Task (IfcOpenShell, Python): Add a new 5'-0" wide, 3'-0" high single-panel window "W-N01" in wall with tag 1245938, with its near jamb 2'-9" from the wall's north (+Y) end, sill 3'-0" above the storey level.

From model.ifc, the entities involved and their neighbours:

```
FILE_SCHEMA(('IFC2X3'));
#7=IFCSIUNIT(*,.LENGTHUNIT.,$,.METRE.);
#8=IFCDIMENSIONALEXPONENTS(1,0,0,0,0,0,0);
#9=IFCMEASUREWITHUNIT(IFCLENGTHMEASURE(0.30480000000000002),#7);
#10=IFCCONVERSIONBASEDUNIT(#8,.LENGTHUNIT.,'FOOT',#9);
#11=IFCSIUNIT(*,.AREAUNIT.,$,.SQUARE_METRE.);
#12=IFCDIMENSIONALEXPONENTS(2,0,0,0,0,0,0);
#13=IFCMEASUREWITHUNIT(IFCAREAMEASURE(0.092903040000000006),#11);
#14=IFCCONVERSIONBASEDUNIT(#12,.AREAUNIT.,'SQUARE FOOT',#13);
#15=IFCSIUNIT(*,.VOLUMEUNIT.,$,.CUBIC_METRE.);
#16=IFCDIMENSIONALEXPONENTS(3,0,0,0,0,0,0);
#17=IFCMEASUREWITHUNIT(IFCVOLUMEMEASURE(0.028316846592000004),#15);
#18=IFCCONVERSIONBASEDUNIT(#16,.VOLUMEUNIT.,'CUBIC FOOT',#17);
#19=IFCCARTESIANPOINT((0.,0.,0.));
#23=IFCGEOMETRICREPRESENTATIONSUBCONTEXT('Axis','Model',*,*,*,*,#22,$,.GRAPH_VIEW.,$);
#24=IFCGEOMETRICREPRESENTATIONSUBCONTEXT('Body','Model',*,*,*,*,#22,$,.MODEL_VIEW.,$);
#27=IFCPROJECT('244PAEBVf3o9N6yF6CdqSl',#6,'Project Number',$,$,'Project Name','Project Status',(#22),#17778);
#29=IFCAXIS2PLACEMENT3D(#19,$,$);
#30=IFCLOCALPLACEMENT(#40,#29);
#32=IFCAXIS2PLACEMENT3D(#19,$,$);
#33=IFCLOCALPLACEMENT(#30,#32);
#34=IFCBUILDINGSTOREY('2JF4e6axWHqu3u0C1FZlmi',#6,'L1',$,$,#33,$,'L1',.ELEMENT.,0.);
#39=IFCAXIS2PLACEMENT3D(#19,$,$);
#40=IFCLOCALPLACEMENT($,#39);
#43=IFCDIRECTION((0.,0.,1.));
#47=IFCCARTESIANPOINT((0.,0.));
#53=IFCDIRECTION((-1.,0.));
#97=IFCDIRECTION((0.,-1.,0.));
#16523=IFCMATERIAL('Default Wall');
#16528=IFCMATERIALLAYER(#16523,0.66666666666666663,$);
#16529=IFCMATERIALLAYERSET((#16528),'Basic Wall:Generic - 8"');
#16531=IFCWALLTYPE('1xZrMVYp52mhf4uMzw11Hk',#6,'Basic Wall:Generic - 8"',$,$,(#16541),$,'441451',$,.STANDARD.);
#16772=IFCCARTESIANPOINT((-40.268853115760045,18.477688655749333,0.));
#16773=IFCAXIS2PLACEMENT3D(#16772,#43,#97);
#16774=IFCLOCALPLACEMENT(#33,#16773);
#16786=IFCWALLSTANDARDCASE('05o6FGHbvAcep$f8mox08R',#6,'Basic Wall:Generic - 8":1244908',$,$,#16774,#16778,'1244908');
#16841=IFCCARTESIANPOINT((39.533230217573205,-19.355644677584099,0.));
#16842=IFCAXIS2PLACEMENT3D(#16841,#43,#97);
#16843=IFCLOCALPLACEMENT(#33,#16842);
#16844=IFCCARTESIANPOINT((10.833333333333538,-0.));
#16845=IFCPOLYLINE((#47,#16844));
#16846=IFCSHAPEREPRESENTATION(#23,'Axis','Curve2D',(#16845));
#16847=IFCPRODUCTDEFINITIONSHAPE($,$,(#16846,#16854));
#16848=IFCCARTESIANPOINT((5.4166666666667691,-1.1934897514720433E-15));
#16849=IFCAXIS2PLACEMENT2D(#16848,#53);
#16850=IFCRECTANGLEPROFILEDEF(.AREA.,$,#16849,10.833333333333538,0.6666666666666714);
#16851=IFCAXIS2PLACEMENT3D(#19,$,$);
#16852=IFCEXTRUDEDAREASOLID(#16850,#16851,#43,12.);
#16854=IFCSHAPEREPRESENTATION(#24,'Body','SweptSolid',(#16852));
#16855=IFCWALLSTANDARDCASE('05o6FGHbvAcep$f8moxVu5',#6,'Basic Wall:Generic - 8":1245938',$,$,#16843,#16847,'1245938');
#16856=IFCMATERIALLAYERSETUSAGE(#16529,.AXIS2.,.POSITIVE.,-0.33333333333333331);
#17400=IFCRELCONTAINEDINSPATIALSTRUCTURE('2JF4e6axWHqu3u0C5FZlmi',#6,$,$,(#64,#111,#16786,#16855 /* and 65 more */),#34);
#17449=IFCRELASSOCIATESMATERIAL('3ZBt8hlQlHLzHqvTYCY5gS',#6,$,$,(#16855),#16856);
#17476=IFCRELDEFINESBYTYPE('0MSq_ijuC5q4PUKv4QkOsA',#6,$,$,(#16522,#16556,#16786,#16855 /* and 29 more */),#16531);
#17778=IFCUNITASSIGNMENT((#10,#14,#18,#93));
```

```python
import numpy as np
import ifcopenshell
import ifcopenshell.api.feature
import ifcopenshell.api.geometry
import ifcopenshell.api.root
import ifcopenshell.api.spatial
import ifcopenshell.api.type
import ifcopenshell.geom
import ifcopenshell.util.element
import ifcopenshell.util.placement
import ifcopenshell.util.representation
import ifcopenshell.util.shape
import ifcopenshell.util.unit

model = ifcopenshell.open("model.ifc")
unit_scale = ifcopenshell.util.unit.calculate_unit_scale(model)
settings = ifcopenshell.geom.settings()


def volume(element):
    """Net volume in cubic metres, openings subtracted."""
    shape = ifcopenshell.geom.create_shape(settings, element)
    return ifcopenshell.util.shape.get_volume(shape.geometry)


wall = model.by_guid("05o6FGHbvAcep$f8moxVu5")
storey = ifcopenshell.util.element.get_container(wall, ifc_class="IfcBuildingStorey")
context = ifcopenshell.util.representation.get_context(model, "Model", "Body", "MODEL_VIEW")
before = volume(wall)

width, height, from_end, sill = 1.524, 0.9144, 0.8382, 0.9144  # metres

# The wall runs along its own X axis, and the end named is its -X end.
wall_shape = ifcopenshell.geom.create_shape(settings, wall)
x, y, z = ifcopenshell.util.shape.get_vertices(wall_shape.geometry).T
start = x.min() + from_end
face, thickness = float(y.min()), float(y.max() - y.min())
wall_matrix = ifcopenshell.util.placement.get_local_placement(wall.ObjectPlacement)
level = ifcopenshell.util.placement.get_local_placement(storey.ObjectPlacement)[2, 3]


def in_wall(x, y):
    """Placement at x, y metres in the wall's axes, at sill height."""
    matrix = wall_matrix.copy()
    matrix[:, 3] = wall_matrix @ np.array([x / unit_scale, y / unit_scale, 0.0, 1.0])
    matrix[2, 3] = level + sill / unit_scale
    return matrix


# Opening: a box that overshoots both wall faces by 50 mm.
opening = ifcopenshell.api.root.create_entity(model, ifc_class="IfcOpeningElement")
box = ifcopenshell.api.geometry.add_wall_representation(
    model, context=context, length=width, height=height, thickness=thickness + 0.1
)
ifcopenshell.api.geometry.assign_representation(model, product=opening, representation=box)
ifcopenshell.api.geometry.edit_object_placement(model, product=opening, matrix=in_wall(start, face - 0.05), is_si=False)
ifcopenshell.api.feature.add_feature(model, feature=opening, element=wall)

window = ifcopenshell.api.root.create_entity(model, ifc_class="IfcWindow", name="W-N01")
window.OverallWidth, window.OverallHeight = width / unit_scale, height / unit_scale
body = ifcopenshell.api.geometry.add_window_representation(
    model,
    context=context,
    overall_width=window.OverallWidth,
    overall_height=window.OverallHeight,
    partition_type="SINGLE_PANEL",
)
ifcopenshell.api.geometry.assign_representation(model, product=window, representation=body)
ifcopenshell.api.spatial.assign_container(model, products=[window], relating_structure=storey)
fills = ifcopenshell.api.feature.add_filling(model, opening=opening, element=window)
fills.OwnerHistory = window.OwnerHistory  # required in IFC2X3

# IFC2X3 keeps the operation on the window style.
style = ifcopenshell.api.root.create_entity(model, ifc_class="IfcWindowStyle", name="W-N01")
style.OperationType, style.ConstructionType = "SINGLE_PANEL", "NOTDEFINED"
style.ParameterTakesPrecedence = style.Sizeable = False
ifcopenshell.api.type.assign_type(model, related_objects=[window], relating_type=style)

# Centre the window in the wall's thickness.
ifcopenshell.api.geometry.edit_object_placement(model, product=window, matrix=in_wall(start, face), is_si=False)
window_shape = ifcopenshell.geom.create_shape(settings, window)
depth = ifcopenshell.util.shape.get_vertices(window_shape.geometry)[:, 1]
offset = face + thickness / 2 - (depth.min() + depth.max()) / 2
ifcopenshell.api.geometry.edit_object_placement(model, product=window, matrix=in_wall(start, offset), is_si=False)

after = volume(wall)

print(f"wall volume {before:.3f} -> {after:.3f} m3")

model.write("model-out.ifc")
```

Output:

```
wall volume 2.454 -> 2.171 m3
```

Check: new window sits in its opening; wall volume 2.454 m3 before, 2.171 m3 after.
